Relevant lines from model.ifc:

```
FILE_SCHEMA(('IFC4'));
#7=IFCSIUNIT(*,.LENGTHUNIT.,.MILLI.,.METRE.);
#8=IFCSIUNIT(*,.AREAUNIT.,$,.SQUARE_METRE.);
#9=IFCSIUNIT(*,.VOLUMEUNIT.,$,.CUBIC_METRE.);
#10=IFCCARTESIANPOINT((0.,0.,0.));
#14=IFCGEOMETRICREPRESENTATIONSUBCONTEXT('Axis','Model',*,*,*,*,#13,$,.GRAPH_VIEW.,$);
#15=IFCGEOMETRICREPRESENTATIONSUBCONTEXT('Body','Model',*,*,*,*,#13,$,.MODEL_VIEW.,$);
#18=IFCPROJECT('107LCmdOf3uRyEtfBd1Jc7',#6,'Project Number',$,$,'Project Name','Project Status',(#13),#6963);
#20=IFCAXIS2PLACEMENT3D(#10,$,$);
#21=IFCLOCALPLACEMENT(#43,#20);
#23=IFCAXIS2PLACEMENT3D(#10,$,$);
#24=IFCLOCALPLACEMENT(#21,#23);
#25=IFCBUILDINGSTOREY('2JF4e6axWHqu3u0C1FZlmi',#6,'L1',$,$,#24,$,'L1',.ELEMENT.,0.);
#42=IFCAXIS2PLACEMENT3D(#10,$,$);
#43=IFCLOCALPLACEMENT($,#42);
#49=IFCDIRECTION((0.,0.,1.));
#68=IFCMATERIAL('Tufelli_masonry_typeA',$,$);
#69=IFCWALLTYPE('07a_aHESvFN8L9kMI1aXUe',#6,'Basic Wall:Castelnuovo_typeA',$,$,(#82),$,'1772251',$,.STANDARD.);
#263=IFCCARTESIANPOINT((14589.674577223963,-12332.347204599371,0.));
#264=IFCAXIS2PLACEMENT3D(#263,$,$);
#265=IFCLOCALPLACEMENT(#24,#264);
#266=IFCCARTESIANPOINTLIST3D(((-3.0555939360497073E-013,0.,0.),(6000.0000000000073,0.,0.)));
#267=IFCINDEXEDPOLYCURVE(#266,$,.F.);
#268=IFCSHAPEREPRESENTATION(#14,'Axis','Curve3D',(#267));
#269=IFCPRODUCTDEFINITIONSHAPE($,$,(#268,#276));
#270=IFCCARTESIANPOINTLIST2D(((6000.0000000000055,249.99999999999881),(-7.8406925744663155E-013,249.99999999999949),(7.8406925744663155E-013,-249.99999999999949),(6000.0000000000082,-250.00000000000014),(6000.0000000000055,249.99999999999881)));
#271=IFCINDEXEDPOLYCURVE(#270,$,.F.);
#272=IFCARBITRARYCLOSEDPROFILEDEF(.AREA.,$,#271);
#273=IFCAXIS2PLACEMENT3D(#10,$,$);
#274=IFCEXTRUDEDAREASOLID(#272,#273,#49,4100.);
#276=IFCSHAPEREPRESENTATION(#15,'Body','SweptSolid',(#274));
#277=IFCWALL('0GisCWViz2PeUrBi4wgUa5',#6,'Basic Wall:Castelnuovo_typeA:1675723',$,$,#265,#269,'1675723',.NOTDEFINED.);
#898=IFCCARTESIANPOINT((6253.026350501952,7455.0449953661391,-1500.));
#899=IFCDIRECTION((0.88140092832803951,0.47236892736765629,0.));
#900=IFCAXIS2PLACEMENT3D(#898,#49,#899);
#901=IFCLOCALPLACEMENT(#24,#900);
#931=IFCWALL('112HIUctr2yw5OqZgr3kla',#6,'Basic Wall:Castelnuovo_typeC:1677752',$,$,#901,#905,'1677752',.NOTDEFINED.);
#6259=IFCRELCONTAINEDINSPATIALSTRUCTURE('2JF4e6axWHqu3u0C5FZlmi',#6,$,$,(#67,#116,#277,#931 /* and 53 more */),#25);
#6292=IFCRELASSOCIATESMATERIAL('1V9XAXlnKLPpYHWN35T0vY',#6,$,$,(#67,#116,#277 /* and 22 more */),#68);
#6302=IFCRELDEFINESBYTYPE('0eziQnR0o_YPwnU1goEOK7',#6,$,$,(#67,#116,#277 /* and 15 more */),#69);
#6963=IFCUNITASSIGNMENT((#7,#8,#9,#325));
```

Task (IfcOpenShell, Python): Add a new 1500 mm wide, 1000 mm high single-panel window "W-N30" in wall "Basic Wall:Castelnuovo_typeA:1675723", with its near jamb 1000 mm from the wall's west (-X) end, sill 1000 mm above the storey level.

```python
import numpy as np
import ifcopenshell
import ifcopenshell.api.feature
import ifcopenshell.api.geometry
import ifcopenshell.api.root
import ifcopenshell.api.spatial
import ifcopenshell.geom
import ifcopenshell.util.element
import ifcopenshell.util.placement
import ifcopenshell.util.representation
import ifcopenshell.util.shape
import ifcopenshell.util.unit

model = ifcopenshell.open("model.ifc")
unit_scale = ifcopenshell.util.unit.calculate_unit_scale(model)
settings = ifcopenshell.geom.settings()


def volume(element):
    """Net volume in cubic metres, openings subtracted."""
    shape = ifcopenshell.geom.create_shape(settings, element)
    return ifcopenshell.util.shape.get_volume(shape.geometry)


wall = model.by_guid("0GisCWViz2PeUrBi4wgUa5")
storey = ifcopenshell.util.element.get_container(wall, ifc_class="IfcBuildingStorey")
context = ifcopenshell.util.representation.get_context(model, "Model", "Body", "MODEL_VIEW")
before = volume(wall)

width, height, from_end, sill = 1.5, 1, 1, 1  # metres

# The wall runs along its own X axis, and the end named is its -X end.
wall_shape = ifcopenshell.geom.create_shape(settings, wall)
x, y, z = ifcopenshell.util.shape.get_vertices(wall_shape.geometry).T
start = x.min() + from_end
face, thickness = float(y.min()), float(y.max() - y.min())
wall_matrix = ifcopenshell.util.placement.get_local_placement(wall.ObjectPlacement)
level = ifcopenshell.util.placement.get_local_placement(storey.ObjectPlacement)[2, 3]


def in_wall(x, y):
    """Placement at x, y metres in the wall's axes, at sill height."""
    matrix = wall_matrix.copy()
    matrix[:, 3] = wall_matrix @ np.array([x / unit_scale, y / unit_scale, 0.0, 1.0])
    matrix[2, 3] = level + sill / unit_scale
    return matrix


# Opening: a box that overshoots both wall faces by 50 mm.
opening = ifcopenshell.api.root.create_entity(model, ifc_class="IfcOpeningElement", predefined_type="OPENING")
box = ifcopenshell.api.geometry.add_wall_representation(
    model, context=context, length=width, height=height, thickness=thickness + 0.1
)
ifcopenshell.api.geometry.assign_representation(model, product=opening, representation=box)
ifcopenshell.api.geometry.edit_object_placement(model, product=opening, matrix=in_wall(start, face - 0.05), is_si=False)
ifcopenshell.api.feature.add_feature(model, feature=opening, element=wall)

window = ifcopenshell.api.root.create_entity(model, ifc_class="IfcWindow", name="W-N30", predefined_type="WINDOW")
window.OverallWidth, window.OverallHeight = width / unit_scale, height / unit_scale
window.PartitioningType = "SINGLE_PANEL"
body = ifcopenshell.api.geometry.add_window_representation(
    model,
    context=context,
    overall_width=window.OverallWidth,
    overall_height=window.OverallHeight,
    partition_type="SINGLE_PANEL",
)
ifcopenshell.api.geometry.assign_representation(model, product=window, representation=body)
ifcopenshell.api.spatial.assign_container(model, products=[window], relating_structure=storey)
ifcopenshell.api.feature.add_filling(model, opening=opening, element=window)

# Centre the window in the wall's thickness.
ifcopenshell.api.geometry.edit_object_placement(model, product=window, matrix=in_wall(start, face), is_si=False)
window_shape = ifcopenshell.geom.create_shape(settings, window)
depth = ifcopenshell.util.shape.get_vertices(window_shape.geometry)[:, 1]
offset = face + thickness / 2 - (depth.min() + depth.max()) / 2
ifcopenshell.api.geometry.edit_object_placement(model, product=window, matrix=in_wall(start, offset), is_si=False)

after = volume(wall)

print(f"wall volume {before:.3f} -> {after:.3f} m3")

model.write("model_edited.ifc")
```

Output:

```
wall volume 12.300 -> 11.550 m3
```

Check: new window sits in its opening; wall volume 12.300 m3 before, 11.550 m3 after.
